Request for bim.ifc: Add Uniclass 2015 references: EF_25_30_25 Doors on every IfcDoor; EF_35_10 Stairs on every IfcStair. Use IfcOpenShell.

First a look at what the model holds.

```python
import ifcopenshell

model = ifcopenshell.open("bim.ifc")
print(model.schema)
print("classifications:", [c.Name for c in model.by_type("IfcClassification")])
for ifc_class in ("IfcDoor", "IfcRoof", "IfcStair", "IfcWall", "IfcWindow"):
    print(ifc_class, len(model.by_type(ifc_class)))
```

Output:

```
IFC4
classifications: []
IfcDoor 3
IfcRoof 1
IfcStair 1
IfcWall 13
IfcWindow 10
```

```python
import ifcopenshell
import ifcopenshell.api.classification

model = ifcopenshell.open("bim.ifc")

system = ifcopenshell.api.classification.add_classification(model, classification="Uniclass 2015")

codes = {
    "IfcDoor": ("EF_25_30_25", "Doors"),
    "IfcStair": ("EF_35_10", "Stairs"),
}
for ifc_class, (code, name) in codes.items():
    products = model.by_type(ifc_class)
    ifcopenshell.api.classification.add_reference(
        model, products=products, classification=system, identification=code, name=name
    )
    print(code, len(products))

model.write("bim_edited.ifc")
```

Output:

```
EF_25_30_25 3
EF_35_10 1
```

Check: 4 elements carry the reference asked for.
